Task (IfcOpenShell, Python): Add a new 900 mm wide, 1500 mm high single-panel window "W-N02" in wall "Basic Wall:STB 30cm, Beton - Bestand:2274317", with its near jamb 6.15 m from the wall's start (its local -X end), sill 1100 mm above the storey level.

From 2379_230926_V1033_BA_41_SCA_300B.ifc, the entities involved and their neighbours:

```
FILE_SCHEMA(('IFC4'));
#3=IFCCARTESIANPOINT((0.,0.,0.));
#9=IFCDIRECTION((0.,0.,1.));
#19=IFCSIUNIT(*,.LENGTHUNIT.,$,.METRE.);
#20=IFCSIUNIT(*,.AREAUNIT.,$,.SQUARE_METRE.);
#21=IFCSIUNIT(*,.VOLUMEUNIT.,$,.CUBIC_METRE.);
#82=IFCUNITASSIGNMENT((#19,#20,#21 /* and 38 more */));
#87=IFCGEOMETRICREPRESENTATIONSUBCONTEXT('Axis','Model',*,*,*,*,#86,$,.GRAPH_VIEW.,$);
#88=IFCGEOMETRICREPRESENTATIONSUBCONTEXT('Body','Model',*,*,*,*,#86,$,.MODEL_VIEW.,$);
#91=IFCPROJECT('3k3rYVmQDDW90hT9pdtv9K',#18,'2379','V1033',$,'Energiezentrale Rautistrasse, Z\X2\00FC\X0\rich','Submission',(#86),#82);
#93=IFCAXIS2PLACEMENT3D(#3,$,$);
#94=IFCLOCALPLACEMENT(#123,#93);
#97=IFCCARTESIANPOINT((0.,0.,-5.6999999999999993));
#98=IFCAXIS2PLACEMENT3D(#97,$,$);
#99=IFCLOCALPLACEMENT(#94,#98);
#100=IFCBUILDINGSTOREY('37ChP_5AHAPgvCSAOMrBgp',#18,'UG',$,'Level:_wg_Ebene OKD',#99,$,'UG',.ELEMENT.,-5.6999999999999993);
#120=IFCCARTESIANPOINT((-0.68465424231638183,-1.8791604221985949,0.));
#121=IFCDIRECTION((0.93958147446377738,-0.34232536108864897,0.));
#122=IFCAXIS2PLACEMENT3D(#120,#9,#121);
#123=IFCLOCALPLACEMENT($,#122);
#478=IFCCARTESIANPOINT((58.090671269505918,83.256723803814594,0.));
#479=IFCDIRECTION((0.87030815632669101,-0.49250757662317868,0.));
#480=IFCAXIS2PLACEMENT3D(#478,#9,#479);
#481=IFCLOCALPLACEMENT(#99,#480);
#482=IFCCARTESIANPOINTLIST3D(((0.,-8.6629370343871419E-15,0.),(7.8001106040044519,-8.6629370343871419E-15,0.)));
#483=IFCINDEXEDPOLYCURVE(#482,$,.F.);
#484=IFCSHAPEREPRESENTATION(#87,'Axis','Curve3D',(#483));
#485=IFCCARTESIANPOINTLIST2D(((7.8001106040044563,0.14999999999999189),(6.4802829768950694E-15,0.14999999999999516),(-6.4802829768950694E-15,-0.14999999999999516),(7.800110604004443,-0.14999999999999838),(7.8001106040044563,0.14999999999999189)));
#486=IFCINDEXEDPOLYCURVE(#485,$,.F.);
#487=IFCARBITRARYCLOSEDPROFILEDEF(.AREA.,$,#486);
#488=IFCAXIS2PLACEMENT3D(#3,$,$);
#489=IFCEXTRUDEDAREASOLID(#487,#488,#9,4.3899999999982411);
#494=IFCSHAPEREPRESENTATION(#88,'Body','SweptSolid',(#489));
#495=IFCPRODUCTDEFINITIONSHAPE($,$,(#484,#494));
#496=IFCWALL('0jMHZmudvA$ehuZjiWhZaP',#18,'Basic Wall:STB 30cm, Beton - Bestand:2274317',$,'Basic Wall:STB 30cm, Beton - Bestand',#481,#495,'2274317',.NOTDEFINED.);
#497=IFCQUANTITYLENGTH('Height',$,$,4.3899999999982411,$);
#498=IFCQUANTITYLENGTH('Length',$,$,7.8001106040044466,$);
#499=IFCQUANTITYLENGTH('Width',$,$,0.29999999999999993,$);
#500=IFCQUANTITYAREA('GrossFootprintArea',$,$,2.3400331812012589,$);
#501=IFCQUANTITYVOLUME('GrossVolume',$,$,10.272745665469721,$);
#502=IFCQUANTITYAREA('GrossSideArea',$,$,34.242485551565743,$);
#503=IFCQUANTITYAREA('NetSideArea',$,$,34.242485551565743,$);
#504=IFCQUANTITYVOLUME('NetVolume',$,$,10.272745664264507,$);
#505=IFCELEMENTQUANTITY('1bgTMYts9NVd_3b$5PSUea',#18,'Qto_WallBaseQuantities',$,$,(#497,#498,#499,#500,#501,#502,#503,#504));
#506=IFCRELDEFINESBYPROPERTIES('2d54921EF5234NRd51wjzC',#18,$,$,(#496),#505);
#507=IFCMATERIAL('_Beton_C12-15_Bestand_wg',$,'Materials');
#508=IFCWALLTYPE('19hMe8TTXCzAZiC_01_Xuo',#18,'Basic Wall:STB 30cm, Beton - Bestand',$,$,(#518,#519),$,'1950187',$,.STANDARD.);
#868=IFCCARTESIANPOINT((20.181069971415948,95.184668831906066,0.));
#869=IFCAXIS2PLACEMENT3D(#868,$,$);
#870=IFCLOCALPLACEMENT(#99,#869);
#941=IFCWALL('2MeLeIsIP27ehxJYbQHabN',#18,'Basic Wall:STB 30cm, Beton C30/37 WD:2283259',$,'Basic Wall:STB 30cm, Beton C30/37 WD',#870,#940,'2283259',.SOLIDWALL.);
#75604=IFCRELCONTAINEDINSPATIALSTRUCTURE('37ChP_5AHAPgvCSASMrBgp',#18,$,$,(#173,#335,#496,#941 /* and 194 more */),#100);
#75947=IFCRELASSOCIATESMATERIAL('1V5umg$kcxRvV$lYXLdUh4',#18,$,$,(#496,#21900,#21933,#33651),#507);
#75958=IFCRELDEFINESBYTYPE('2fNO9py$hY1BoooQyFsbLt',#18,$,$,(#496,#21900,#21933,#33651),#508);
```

```python
import numpy as np
import ifcopenshell
import ifcopenshell.api.feature
import ifcopenshell.api.geometry
import ifcopenshell.api.pset
import ifcopenshell.api.root
import ifcopenshell.api.spatial
import ifcopenshell.geom
import ifcopenshell.util.element
import ifcopenshell.util.placement
import ifcopenshell.util.representation
import ifcopenshell.util.shape
import ifcopenshell.util.unit

model = ifcopenshell.open("2379_230926_V1033_BA_41_SCA_300B.ifc")
unit_scale = ifcopenshell.util.unit.calculate_unit_scale(model)
area_scale = ifcopenshell.util.unit.calculate_unit_scale(model, "AREAUNIT")
volume_scale = ifcopenshell.util.unit.calculate_unit_scale(model, "VOLUMEUNIT")
settings = ifcopenshell.geom.settings()


def volume(element):
    """Net volume in cubic metres, openings subtracted."""
    shape = ifcopenshell.geom.create_shape(settings, element)
    return ifcopenshell.util.shape.get_volume(shape.geometry)


wall = model.by_guid("0jMHZmudvA$ehuZjiWhZaP")
storey = ifcopenshell.util.element.get_container(wall, ifc_class="IfcBuildingStorey")
context = ifcopenshell.util.representation.get_context(model, "Model", "Body", "MODEL_VIEW")
before = volume(wall)

width, height, from_end, sill = 0.9, 1.5, 6.15, 1.1  # metres

# The wall runs along its own X axis, and the end named is its -X end.
wall_shape = ifcopenshell.geom.create_shape(settings, wall)
x, y, z = ifcopenshell.util.shape.get_vertices(wall_shape.geometry).T
start = x.min() + from_end
face, thickness = float(y.min()), float(y.max() - y.min())
wall_matrix = ifcopenshell.util.placement.get_local_placement(wall.ObjectPlacement)
level = ifcopenshell.util.placement.get_local_placement(storey.ObjectPlacement)[2, 3]


def in_wall(x, y):
    """Placement at x, y metres in the wall's axes, at sill height."""
    matrix = wall_matrix.copy()
    matrix[:, 3] = wall_matrix @ np.array([x / unit_scale, y / unit_scale, 0.0, 1.0])
    matrix[2, 3] = level + sill / unit_scale
    return matrix


# Opening: a box that overshoots both wall faces by 50 mm.
opening = ifcopenshell.api.root.create_entity(model, ifc_class="IfcOpeningElement", predefined_type="OPENING")
box = ifcopenshell.api.geometry.add_wall_representation(
    model, context=context, length=width, height=height, thickness=thickness + 0.1
)
ifcopenshell.api.geometry.assign_representation(model, product=opening, representation=box)
ifcopenshell.api.geometry.edit_object_placement(model, product=opening, matrix=in_wall(start, face - 0.05), is_si=False)
ifcopenshell.api.feature.add_feature(model, feature=opening, element=wall)

window = ifcopenshell.api.root.create_entity(model, ifc_class="IfcWindow", name="W-N02", predefined_type="WINDOW")
window.OverallWidth, window.OverallHeight = width / unit_scale, height / unit_scale
window.PartitioningType = "SINGLE_PANEL"
body = ifcopenshell.api.geometry.add_window_representation(
    model,
    context=context,
    overall_width=window.OverallWidth,
    overall_height=window.OverallHeight,
    partition_type="SINGLE_PANEL",
)
ifcopenshell.api.geometry.assign_representation(model, product=window, representation=body)
ifcopenshell.api.spatial.assign_container(model, products=[window], relating_structure=storey)
ifcopenshell.api.feature.add_filling(model, opening=opening, element=window)

# Centre the window in the wall's thickness.
ifcopenshell.api.geometry.edit_object_placement(model, product=window, matrix=in_wall(start, face), is_si=False)
window_shape = ifcopenshell.geom.create_shape(settings, window)
depth = ifcopenshell.util.shape.get_vertices(window_shape.geometry)[:, 1]
offset = face + thickness / 2 - (depth.min() + depth.max()) / 2
ifcopenshell.api.geometry.edit_object_placement(model, product=window, matrix=in_wall(start, offset), is_si=False)

after = volume(wall)

# Update the wall's stored quantities.
qto = model.by_id(ifcopenshell.util.element.get_pset(wall, "Qto_WallBaseQuantities", should_inherit=False)["id"])
ifcopenshell.api.pset.edit_qto(model, qto=qto, properties={
    "NetSideArea": after / thickness / area_scale,
    "NetVolume": after / volume_scale,
})

print(f"wall volume {before:.3f} -> {after:.3f} m3")

model.write("2379_230926_V1033_BA_41_SCA_300B_updated.ifc")
```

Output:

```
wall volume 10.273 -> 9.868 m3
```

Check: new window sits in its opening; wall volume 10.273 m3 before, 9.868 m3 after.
